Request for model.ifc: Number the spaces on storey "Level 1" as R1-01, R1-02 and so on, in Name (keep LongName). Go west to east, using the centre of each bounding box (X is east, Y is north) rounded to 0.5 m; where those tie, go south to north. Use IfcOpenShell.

First a look at what the model holds.

```python
import ifcopenshell
import ifcopenshell.util.element
import ifcopenshell.util.placement

model = ifcopenshell.open("model.ifc")
print(model.schema)
storey = next(s for s in model.by_type("IfcBuildingStorey") if s.Name == "Level 1")
spaces = [e for e in ifcopenshell.util.element.get_decomposition(storey) if e.is_a("IfcSpace")]
for e in sorted(spaces, key=lambda e: e.id()):
    origin = ifcopenshell.util.placement.get_local_placement(e.ObjectPlacement)[:3, 3]
    print(e.id(), e.Name, e.LongName, origin.round(2) + 0.0, sep=" | ")
```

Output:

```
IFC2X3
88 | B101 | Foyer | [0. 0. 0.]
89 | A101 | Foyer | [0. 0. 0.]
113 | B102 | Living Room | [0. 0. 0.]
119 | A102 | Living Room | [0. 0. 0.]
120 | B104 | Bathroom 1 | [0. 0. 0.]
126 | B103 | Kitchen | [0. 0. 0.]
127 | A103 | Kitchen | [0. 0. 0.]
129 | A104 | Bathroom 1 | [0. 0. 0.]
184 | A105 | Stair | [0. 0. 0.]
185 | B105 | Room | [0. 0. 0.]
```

```python
import ifcopenshell
import ifcopenshell.geom
import ifcopenshell.util.element
import ifcopenshell.util.shape

model = ifcopenshell.open("model.ifc")
settings = ifcopenshell.geom.settings()
settings.set("use-world-coords", True)


def centre(element):
    shape = ifcopenshell.geom.create_shape(settings, element)
    return ifcopenshell.util.shape.get_bbox_centroid(shape.geometry)


storey = next(s for s in model.by_type("IfcBuildingStorey") if s.Name == "Level 1")
spaces = [e for e in ifcopenshell.util.element.get_decomposition(storey) if e.is_a("IfcSpace")]

# Insertion points can sit at a corner or the storey origin, so sort by the geometry (in metres).
centres = {e: centre(e) for e in spaces}
spaces.sort(key=lambda e: (round(centres[e][0] / 0.5), centres[e][1]))

for i, e in enumerate(spaces, start=1):
    number = f"R1-{i:02d}"
    e.Name = number
    print(e.id(), number)

model.write("model_v2.ifc")
```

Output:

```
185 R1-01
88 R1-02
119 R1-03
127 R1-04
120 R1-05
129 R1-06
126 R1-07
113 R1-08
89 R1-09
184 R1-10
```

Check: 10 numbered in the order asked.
